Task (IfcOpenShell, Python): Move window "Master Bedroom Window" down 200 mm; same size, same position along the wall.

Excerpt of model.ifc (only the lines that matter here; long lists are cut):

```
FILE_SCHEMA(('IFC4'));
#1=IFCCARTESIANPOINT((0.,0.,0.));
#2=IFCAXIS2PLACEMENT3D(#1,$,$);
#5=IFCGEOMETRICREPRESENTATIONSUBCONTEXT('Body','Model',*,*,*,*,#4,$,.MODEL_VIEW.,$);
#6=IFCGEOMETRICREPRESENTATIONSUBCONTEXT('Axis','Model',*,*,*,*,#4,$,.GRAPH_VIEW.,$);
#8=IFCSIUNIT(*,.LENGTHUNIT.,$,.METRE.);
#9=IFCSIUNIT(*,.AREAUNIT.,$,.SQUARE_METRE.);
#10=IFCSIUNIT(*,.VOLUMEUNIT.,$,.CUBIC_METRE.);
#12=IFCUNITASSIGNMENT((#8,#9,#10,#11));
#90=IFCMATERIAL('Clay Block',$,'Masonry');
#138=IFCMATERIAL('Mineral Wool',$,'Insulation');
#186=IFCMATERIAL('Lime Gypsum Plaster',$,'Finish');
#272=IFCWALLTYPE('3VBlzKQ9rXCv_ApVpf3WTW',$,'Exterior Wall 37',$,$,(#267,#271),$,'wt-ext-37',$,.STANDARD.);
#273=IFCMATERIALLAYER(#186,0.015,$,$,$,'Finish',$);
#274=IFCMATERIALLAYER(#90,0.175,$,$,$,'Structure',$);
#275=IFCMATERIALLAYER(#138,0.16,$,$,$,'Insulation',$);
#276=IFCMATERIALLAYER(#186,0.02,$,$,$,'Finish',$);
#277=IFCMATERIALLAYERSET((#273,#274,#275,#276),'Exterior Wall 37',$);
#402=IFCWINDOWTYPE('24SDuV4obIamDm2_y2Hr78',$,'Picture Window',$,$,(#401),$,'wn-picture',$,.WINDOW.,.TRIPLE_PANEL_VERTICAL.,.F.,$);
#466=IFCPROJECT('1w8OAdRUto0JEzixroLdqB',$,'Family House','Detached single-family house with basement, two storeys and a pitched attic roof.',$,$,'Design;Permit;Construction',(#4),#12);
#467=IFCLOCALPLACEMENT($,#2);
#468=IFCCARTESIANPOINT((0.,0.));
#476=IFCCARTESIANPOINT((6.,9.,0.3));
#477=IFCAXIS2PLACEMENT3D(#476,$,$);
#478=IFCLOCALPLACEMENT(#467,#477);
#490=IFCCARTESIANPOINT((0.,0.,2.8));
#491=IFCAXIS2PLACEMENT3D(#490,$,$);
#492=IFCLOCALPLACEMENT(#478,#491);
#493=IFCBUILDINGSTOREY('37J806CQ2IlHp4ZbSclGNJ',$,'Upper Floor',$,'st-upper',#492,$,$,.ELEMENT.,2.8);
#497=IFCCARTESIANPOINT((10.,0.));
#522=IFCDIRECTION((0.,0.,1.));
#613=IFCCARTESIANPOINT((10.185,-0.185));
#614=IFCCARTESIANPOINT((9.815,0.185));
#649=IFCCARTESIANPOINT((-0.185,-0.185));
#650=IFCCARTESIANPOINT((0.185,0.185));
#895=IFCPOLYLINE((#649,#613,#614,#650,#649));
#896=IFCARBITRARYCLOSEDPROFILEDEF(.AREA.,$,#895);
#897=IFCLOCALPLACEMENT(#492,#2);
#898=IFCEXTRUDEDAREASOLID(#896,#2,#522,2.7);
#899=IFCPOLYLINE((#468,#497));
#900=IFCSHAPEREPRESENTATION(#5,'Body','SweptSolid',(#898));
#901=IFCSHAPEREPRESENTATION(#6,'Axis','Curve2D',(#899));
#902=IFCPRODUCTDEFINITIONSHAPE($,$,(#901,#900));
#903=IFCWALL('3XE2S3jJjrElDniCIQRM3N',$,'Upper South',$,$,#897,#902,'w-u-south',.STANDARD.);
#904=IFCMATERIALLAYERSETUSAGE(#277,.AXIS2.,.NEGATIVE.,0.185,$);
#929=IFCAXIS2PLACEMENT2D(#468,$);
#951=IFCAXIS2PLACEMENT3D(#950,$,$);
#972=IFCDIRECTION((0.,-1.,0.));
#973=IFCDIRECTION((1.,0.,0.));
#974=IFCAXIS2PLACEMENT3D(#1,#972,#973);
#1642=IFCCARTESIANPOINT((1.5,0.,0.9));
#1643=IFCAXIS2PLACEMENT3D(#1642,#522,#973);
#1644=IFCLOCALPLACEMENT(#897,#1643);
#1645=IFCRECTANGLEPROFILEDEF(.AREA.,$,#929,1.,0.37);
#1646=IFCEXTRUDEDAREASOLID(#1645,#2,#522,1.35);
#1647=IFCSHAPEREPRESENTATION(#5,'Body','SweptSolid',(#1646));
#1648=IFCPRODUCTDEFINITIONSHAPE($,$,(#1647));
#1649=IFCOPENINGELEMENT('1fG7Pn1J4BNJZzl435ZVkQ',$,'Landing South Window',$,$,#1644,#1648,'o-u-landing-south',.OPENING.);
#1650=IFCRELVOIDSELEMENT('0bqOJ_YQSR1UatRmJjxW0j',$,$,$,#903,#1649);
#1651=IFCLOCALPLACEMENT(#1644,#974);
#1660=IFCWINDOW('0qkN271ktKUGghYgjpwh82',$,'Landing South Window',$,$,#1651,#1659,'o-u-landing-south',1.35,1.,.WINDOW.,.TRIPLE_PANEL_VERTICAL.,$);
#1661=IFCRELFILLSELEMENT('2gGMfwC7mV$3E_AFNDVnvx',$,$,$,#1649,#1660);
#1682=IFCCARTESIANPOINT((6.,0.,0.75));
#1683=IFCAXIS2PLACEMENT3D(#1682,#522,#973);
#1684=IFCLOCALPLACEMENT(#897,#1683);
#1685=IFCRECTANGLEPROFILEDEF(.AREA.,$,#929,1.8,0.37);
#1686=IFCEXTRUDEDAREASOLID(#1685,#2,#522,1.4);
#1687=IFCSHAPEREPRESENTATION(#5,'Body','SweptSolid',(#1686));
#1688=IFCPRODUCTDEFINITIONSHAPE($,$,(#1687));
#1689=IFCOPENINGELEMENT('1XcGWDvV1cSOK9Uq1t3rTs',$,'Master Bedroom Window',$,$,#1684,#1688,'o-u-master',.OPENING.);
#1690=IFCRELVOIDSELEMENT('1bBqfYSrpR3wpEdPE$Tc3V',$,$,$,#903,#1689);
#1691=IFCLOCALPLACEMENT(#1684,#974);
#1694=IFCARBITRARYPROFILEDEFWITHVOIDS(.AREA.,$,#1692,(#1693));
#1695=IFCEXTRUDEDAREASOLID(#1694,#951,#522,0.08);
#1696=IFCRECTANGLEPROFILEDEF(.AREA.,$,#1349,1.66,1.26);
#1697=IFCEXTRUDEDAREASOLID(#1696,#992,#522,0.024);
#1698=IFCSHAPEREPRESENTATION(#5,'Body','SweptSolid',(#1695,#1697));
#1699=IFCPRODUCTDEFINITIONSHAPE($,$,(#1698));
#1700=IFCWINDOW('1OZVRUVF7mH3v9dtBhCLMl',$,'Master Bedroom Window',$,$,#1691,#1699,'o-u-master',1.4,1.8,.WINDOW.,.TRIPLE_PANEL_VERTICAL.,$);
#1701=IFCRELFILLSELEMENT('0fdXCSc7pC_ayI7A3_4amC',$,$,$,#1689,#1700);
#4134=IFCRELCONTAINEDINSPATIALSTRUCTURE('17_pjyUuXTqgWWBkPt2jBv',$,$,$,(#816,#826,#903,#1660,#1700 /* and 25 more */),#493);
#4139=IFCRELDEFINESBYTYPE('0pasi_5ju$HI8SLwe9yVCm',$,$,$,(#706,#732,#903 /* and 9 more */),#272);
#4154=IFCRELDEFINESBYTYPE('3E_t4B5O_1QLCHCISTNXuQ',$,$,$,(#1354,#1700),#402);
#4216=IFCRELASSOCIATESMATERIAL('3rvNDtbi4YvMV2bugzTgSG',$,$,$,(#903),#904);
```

```python
import numpy as np
import ifcopenshell
import ifcopenshell.api.geometry
import ifcopenshell.util.placement
import ifcopenshell.util.unit

model = ifcopenshell.open("model.ifc")
unit_scale = ifcopenshell.util.unit.calculate_unit_scale(model)

window = model.by_guid("1OZVRUVF7mH3v9dtBhCLMl")
opening = window.FillsVoids[0].RelatingOpeningElement
dz = -0.2 / unit_scale

shift = np.array([0.0, 0.0, dz])
# The window is placed relative to its opening, so it follows when the opening moves.
matrix = ifcopenshell.util.placement.get_local_placement(opening.ObjectPlacement)
matrix[:3, 3] += shift
ifcopenshell.api.geometry.edit_object_placement(
    model, product=opening, matrix=matrix, is_si=False, should_transform_children=True
)

print(f"moved by {dz * unit_scale:+.3f} m")

model.write("model_edited.ifc")
```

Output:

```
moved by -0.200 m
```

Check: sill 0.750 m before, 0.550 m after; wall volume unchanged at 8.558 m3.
